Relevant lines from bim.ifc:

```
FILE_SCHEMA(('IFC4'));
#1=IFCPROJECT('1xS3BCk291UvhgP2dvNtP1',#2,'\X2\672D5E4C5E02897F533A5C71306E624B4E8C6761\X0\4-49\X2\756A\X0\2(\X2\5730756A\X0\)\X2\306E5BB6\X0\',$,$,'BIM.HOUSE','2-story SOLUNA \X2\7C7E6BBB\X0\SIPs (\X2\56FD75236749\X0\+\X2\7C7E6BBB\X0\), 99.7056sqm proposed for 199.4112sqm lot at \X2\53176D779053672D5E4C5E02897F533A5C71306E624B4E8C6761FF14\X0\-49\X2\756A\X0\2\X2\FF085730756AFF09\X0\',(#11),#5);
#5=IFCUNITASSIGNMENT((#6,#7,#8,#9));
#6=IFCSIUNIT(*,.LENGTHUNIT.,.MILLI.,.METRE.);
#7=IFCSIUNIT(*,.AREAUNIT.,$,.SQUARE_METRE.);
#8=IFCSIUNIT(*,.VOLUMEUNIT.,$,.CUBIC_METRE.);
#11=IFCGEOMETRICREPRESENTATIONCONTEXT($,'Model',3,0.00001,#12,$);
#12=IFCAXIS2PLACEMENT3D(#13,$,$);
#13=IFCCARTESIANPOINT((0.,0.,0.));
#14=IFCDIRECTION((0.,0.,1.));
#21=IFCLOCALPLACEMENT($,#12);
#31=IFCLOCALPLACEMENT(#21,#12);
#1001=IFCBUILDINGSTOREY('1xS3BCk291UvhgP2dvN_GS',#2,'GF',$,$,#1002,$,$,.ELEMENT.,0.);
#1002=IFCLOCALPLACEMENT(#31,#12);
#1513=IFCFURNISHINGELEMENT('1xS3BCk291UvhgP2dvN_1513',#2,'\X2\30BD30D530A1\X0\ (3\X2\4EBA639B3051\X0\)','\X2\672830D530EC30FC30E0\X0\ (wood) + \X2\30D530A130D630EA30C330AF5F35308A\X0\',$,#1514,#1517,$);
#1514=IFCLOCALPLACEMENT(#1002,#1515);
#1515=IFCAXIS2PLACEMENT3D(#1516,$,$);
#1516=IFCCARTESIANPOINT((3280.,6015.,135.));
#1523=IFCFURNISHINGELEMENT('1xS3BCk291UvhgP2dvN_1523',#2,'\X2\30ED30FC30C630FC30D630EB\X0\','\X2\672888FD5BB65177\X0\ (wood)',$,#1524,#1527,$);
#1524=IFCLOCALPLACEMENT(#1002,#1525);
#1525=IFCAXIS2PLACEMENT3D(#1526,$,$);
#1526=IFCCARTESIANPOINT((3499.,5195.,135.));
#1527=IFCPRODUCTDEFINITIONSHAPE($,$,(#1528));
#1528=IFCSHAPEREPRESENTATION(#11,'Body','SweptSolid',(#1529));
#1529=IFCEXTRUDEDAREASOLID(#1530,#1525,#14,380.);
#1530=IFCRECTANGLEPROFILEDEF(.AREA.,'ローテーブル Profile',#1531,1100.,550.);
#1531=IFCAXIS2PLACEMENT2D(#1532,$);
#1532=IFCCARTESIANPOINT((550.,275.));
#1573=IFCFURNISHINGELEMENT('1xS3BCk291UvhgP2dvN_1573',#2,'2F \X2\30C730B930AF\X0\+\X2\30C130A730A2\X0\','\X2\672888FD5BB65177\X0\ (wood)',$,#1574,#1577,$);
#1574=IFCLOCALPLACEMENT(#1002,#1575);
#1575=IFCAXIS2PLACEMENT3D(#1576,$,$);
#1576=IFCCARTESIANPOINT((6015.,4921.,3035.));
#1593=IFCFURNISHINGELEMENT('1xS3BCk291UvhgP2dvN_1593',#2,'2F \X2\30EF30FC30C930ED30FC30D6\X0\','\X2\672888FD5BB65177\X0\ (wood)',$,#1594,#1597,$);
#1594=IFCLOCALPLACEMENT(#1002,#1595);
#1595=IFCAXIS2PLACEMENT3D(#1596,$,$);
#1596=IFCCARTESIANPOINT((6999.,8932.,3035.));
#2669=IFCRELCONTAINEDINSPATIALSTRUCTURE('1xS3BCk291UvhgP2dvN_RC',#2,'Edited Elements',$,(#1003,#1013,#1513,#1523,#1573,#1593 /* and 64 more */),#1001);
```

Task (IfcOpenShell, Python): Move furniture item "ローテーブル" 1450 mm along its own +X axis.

```python
import ifcopenshell
import ifcopenshell.api.geometry
import ifcopenshell.util.placement
import ifcopenshell.util.unit

model = ifcopenshell.open("bim.ifc")
unit_scale = ifcopenshell.util.unit.calculate_unit_scale(model)

item = model.by_guid("1xS3BCk291UvhgP2dvN_1523")
matrix = ifcopenshell.util.placement.get_local_placement(item.ObjectPlacement)
matrix[:3, 3] += matrix[:3, 0] * 1.45 / unit_scale
ifcopenshell.api.geometry.edit_object_placement(model, product=item, matrix=matrix, is_si=False)

print(ifcopenshell.util.placement.get_local_placement(item.ObjectPlacement).round(3) + 0.0)

model.write("bim_edited.ifc")
```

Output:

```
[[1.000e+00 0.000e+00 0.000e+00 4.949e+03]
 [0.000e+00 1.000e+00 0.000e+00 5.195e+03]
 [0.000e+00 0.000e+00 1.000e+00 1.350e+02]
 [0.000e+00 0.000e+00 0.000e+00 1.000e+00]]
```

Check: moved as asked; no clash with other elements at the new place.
